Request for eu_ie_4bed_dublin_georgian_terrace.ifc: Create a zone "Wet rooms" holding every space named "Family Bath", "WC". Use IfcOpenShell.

First a look at what the model holds.

```python
import ifcopenshell

model = ifcopenshell.open("eu_ie_4bed_dublin_georgian_terrace.ifc")
print(model.schema)
seen = {}
for space in model.by_type("IfcSpace"):
    seen[space.LongName] = seen.get(space.LongName, 0) + 1
for name, count in sorted(seen.items(), key=str):
    print(count, "x", name)
print("zones:", [z.Name for z in model.by_type("IfcZone")][:20])
```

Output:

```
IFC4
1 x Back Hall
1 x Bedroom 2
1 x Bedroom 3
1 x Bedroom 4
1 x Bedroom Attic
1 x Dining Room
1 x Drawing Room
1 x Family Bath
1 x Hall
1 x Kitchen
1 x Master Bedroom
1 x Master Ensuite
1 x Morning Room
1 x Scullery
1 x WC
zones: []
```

```python
import ifcopenshell
import ifcopenshell.api.group
import ifcopenshell.api.root

model = ifcopenshell.open("eu_ie_4bed_dublin_georgian_terrace.ifc")

names = {"Family Bath", "WC"}
spaces = [s for s in model.by_type("IfcSpace") if s.LongName in names]

zone = ifcopenshell.api.root.create_entity(model, ifc_class="IfcZone", name="Wet rooms")
ifcopenshell.api.group.assign_group(model, products=spaces, group=zone)
print(len(spaces), "spaces in", zone.Name)

model.write("eu_ie_4bed_dublin_georgian_terrace_v2.ifc")
```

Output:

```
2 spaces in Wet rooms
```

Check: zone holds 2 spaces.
